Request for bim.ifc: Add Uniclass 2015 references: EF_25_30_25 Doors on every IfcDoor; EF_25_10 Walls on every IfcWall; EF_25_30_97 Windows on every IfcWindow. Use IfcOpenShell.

First a look at what the model holds.

```python
import ifcopenshell

model = ifcopenshell.open("bim.ifc")
print(model.schema)
print("classifications:", [c.Name for c in model.by_type("IfcClassification")])
for ifc_class in ("IfcDoor", "IfcRoof", "IfcStair", "IfcWall", "IfcWindow"):
    print(ifc_class, len(model.by_type(ifc_class)))
```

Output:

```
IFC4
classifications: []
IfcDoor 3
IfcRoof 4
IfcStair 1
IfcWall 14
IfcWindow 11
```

```python
import ifcopenshell
import ifcopenshell.api.classification

model = ifcopenshell.open("bim.ifc")

system = ifcopenshell.api.classification.add_classification(model, classification="Uniclass 2015")

codes = {
    "IfcDoor": ("EF_25_30_25", "Doors"),
    "IfcWall": ("EF_25_10", "Walls"),
    "IfcWindow": ("EF_25_30_97", "Windows"),
}
for ifc_class, (code, name) in codes.items():
    products = model.by_type(ifc_class)
    ifcopenshell.api.classification.add_reference(
        model, products=products, classification=system, identification=code, name=name
    )
    print(code, len(products))

model.write("bim_rev.ifc")
```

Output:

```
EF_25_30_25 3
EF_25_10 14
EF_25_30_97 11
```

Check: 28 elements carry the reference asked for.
